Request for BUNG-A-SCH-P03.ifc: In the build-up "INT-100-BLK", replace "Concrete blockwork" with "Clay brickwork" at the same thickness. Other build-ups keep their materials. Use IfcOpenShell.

First a look at what the model holds.

```python
import ifcopenshell
import ifcopenshell.util.element

model = ifcopenshell.open("BUNG-A-SCH-P03.ifc")
print(model.schema)
for layer_set in model.by_type("IfcMaterialLayerSet"):
    if layer_set.LayerSetName == "INT-100-BLK":
        for layer in layer_set.MaterialLayers:
            print(layer.id(), layer.Material and layer.Material.Name, layer.LayerThickness, sep=" | ")
        print(len(ifcopenshell.util.element.get_elements_by_material(model, layer_set)), "elements and types use it")
print(sorted(m.Name for m in model.by_type("IfcMaterial") if m.Name)[:60])
```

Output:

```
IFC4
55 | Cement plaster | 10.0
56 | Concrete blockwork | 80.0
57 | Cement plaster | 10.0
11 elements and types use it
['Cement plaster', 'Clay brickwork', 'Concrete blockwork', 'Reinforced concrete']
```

```python
import ifcopenshell
import ifcopenshell.api.material

model = ifcopenshell.open("BUNG-A-SCH-P03.ifc")

layer_set = next(s for s in model.by_type("IfcMaterialLayerSet") if s.LayerSetName == "INT-100-BLK")
layer = next(l for l in layer_set.MaterialLayers if l.Material and l.Material.Name == "Concrete blockwork")
material = next(m for m in model.by_type("IfcMaterial") if m.Name == "Clay brickwork")

# Point this one layer at the other material; renaming the old one would change it everywhere.
ifcopenshell.api.material.edit_layer(model, layer=layer, attributes={"Name": material.Name}, material=material)

print([l.Material.Name if l.Material else None for l in layer_set.MaterialLayers])

model.write("BUNG-A-SCH-P03_updated.ifc")
```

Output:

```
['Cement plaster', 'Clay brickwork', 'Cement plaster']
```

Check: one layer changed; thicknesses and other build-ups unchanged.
